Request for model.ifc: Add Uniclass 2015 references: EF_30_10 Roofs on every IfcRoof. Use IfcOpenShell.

First a look at what the model holds.

```python
import ifcopenshell

model = ifcopenshell.open("model.ifc")
print(model.schema)
print("classifications:", [c.Name for c in model.by_type("IfcClassification")])
for ifc_class in ("IfcDoor", "IfcRoof", "IfcStair", "IfcWall", "IfcWindow"):
    print(ifc_class, len(model.by_type(ifc_class)))
```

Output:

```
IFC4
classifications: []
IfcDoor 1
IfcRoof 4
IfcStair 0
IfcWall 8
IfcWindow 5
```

```python
import ifcopenshell
import ifcopenshell.api.classification

model = ifcopenshell.open("model.ifc")

system = ifcopenshell.api.classification.add_classification(model, classification="Uniclass 2015")

codes = {
    "IfcRoof": ("EF_30_10", "Roofs"),
}
for ifc_class, (code, name) in codes.items():
    products = model.by_type(ifc_class)
    ifcopenshell.api.classification.add_reference(
        model, products=products, classification=system, identification=code, name=name
    )
    print(code, len(products))

model.write("model-out.ifc")
```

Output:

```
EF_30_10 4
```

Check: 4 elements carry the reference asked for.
